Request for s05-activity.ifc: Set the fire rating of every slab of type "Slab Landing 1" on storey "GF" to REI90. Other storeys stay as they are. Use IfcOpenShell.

First a look at what the model holds.

```python
import ifcopenshell
import ifcopenshell.util.element

model = ifcopenshell.open("s05-activity.ifc")
print(model.schema)
storey = next(s for s in model.by_type("IfcBuildingStorey") if s.Name == "GF")
slabs = [e for e in ifcopenshell.util.element.get_decomposition(storey) if e.is_a("IfcSlab")]
seen = {}
for e in slabs:
    element_type = ifcopenshell.util.element.get_type(e)
    key = (element_type.Name if element_type != e and element_type else None, ifcopenshell.util.element.get_pset(e, "Pset_SlabCommon", "FireRating"))
    seen[key] = seen.get(key, 0) + 1
for (name, value), count in sorted(seen.items(), key=str):
    print(count, "x", name, "|", value)
```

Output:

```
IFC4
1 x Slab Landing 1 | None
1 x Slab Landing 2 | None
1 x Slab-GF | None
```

```python
import ifcopenshell
import ifcopenshell.api.pset
import ifcopenshell.util.element

model = ifcopenshell.open("s05-activity.ifc")

storey = next(s for s in model.by_type("IfcBuildingStorey") if s.Name == "GF")
slabs = [e for e in ifcopenshell.util.element.get_decomposition(storey) if e.is_a("IfcSlab")]

count = 0
for e in slabs:
    element_type = ifcopenshell.util.element.get_type(e)
    if element_type in (None, e) or element_type.Name != "Slab Landing 1":
        continue
    # add_pset returns the element's existing set when there is one.
    pset = ifcopenshell.api.pset.add_pset(model, product=e, name="Pset_SlabCommon")
    ifcopenshell.api.pset.edit_pset(model, pset=pset, properties={"FireRating": "REI90"})
    count += 1

print(count, "slabs updated")

model.write("s05-activity_v2.ifc")
```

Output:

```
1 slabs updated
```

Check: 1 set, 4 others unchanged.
